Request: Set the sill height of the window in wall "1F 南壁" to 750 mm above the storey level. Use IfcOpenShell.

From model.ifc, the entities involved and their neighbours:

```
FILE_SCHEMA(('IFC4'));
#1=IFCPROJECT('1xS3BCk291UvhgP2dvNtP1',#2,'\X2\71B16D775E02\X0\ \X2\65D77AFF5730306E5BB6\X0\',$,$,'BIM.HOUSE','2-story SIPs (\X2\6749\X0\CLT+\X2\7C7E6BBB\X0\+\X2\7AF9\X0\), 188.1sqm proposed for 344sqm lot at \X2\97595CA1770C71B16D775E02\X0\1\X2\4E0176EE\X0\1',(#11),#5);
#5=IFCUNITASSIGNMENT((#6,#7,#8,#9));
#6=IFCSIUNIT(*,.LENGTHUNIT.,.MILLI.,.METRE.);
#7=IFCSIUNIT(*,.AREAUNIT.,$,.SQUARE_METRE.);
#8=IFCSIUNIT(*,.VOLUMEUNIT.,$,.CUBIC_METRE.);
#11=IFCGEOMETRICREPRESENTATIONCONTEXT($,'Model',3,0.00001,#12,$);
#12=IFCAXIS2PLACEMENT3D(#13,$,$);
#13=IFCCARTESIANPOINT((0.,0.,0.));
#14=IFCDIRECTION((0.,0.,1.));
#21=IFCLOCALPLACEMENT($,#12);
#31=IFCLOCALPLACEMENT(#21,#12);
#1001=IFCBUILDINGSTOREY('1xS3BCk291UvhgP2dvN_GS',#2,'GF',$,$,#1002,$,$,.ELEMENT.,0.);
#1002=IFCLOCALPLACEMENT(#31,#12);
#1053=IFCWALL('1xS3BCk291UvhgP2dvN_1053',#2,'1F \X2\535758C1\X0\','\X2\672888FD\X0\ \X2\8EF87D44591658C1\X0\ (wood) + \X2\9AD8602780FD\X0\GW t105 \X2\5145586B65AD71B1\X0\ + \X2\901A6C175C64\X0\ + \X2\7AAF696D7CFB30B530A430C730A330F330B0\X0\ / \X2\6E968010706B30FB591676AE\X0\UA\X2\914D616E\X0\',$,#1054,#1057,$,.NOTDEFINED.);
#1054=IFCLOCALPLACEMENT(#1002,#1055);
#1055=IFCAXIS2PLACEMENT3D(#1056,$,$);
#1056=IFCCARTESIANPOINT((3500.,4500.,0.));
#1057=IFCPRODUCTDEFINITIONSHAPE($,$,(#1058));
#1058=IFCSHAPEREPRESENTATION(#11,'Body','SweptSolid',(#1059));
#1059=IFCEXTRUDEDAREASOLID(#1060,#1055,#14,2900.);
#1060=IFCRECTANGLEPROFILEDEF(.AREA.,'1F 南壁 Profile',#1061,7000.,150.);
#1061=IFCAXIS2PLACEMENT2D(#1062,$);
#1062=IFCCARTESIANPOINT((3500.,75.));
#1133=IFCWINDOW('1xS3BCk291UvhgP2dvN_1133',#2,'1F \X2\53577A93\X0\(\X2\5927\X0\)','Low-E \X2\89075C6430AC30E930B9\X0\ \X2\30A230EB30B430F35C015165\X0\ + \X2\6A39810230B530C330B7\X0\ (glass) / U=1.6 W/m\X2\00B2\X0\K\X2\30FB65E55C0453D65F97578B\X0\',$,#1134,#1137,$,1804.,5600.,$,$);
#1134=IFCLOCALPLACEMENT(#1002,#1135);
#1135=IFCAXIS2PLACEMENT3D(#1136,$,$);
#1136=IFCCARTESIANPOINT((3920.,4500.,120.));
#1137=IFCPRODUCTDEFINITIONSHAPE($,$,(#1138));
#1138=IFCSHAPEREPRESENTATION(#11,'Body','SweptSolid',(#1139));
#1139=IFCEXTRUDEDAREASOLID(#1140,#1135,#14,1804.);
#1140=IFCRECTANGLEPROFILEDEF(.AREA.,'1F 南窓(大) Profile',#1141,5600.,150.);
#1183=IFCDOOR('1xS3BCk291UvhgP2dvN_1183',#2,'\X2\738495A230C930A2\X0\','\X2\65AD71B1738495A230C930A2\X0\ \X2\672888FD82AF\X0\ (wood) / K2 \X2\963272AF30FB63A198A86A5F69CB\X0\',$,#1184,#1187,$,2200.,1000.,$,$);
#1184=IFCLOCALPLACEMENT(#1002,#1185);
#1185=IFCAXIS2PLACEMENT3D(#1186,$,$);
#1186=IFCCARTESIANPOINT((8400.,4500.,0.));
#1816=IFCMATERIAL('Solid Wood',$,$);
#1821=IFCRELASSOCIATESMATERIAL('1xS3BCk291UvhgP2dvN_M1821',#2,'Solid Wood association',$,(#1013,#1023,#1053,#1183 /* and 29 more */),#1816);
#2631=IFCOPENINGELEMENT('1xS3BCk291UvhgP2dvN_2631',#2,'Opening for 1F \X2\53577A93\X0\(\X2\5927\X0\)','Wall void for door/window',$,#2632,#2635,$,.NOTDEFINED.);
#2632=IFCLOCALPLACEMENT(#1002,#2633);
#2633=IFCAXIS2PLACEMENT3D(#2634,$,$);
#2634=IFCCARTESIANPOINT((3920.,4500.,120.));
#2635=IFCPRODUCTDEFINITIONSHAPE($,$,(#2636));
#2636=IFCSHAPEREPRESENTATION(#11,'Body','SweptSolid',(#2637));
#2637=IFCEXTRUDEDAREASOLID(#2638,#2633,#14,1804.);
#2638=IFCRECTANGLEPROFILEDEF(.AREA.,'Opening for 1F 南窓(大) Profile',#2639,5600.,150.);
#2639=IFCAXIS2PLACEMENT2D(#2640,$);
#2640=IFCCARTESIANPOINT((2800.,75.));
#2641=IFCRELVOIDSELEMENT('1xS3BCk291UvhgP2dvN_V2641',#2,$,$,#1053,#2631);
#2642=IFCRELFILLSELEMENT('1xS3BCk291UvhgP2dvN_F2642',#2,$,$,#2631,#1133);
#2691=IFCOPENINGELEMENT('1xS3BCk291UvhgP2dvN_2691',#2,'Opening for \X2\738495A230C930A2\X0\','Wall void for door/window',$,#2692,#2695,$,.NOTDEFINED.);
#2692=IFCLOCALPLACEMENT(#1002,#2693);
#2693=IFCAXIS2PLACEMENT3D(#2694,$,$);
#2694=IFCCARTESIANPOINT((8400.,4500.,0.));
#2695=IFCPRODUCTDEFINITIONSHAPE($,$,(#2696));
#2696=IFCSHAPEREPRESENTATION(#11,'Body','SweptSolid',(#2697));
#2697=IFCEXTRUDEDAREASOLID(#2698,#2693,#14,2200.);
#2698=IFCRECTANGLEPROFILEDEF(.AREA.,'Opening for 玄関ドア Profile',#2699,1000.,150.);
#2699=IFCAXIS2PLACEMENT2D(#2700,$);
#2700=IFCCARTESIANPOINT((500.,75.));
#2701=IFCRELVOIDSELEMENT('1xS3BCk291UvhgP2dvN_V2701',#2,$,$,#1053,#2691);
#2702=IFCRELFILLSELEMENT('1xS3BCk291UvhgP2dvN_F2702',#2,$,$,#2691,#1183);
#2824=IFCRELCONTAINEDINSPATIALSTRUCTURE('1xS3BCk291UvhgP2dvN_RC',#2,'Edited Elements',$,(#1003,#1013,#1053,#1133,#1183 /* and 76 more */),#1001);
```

```python
import numpy as np
import ifcopenshell
import ifcopenshell.api.geometry
import ifcopenshell.geom
import ifcopenshell.util.element
import ifcopenshell.util.placement
import ifcopenshell.util.shape
import ifcopenshell.util.unit

model = ifcopenshell.open("model.ifc")
unit_scale = ifcopenshell.util.unit.calculate_unit_scale(model)

window = model.by_id(1133)
opening = window.FillsVoids[0].RelatingOpeningElement
storey = ifcopenshell.util.element.get_container(window, ifc_class="IfcBuildingStorey")
level = ifcopenshell.util.placement.get_local_placement(storey.ObjectPlacement)[2, 3]

# The opening's origin need not be at the sill, so measure its lowest point.
shape = ifcopenshell.geom.create_shape(ifcopenshell.geom.settings(), opening)
bottom = ifcopenshell.util.shape.get_shape_bottom_elevation(shape, shape.geometry) / unit_scale
dz = level + 0.75 / unit_scale - bottom

shift = np.array([0.0, 0.0, dz])
# The window is not placed relative to its opening, so move both.
for product in (opening, window):
    matrix = ifcopenshell.util.placement.get_local_placement(product.ObjectPlacement)
    matrix[:3, 3] += shift
    ifcopenshell.api.geometry.edit_object_placement(model, product=product, matrix=matrix, is_si=False)

print(f"moved by {dz * unit_scale:+.3f} m")

model.write("model_rev.ifc")
```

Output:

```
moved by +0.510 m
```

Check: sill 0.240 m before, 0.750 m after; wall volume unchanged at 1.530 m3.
